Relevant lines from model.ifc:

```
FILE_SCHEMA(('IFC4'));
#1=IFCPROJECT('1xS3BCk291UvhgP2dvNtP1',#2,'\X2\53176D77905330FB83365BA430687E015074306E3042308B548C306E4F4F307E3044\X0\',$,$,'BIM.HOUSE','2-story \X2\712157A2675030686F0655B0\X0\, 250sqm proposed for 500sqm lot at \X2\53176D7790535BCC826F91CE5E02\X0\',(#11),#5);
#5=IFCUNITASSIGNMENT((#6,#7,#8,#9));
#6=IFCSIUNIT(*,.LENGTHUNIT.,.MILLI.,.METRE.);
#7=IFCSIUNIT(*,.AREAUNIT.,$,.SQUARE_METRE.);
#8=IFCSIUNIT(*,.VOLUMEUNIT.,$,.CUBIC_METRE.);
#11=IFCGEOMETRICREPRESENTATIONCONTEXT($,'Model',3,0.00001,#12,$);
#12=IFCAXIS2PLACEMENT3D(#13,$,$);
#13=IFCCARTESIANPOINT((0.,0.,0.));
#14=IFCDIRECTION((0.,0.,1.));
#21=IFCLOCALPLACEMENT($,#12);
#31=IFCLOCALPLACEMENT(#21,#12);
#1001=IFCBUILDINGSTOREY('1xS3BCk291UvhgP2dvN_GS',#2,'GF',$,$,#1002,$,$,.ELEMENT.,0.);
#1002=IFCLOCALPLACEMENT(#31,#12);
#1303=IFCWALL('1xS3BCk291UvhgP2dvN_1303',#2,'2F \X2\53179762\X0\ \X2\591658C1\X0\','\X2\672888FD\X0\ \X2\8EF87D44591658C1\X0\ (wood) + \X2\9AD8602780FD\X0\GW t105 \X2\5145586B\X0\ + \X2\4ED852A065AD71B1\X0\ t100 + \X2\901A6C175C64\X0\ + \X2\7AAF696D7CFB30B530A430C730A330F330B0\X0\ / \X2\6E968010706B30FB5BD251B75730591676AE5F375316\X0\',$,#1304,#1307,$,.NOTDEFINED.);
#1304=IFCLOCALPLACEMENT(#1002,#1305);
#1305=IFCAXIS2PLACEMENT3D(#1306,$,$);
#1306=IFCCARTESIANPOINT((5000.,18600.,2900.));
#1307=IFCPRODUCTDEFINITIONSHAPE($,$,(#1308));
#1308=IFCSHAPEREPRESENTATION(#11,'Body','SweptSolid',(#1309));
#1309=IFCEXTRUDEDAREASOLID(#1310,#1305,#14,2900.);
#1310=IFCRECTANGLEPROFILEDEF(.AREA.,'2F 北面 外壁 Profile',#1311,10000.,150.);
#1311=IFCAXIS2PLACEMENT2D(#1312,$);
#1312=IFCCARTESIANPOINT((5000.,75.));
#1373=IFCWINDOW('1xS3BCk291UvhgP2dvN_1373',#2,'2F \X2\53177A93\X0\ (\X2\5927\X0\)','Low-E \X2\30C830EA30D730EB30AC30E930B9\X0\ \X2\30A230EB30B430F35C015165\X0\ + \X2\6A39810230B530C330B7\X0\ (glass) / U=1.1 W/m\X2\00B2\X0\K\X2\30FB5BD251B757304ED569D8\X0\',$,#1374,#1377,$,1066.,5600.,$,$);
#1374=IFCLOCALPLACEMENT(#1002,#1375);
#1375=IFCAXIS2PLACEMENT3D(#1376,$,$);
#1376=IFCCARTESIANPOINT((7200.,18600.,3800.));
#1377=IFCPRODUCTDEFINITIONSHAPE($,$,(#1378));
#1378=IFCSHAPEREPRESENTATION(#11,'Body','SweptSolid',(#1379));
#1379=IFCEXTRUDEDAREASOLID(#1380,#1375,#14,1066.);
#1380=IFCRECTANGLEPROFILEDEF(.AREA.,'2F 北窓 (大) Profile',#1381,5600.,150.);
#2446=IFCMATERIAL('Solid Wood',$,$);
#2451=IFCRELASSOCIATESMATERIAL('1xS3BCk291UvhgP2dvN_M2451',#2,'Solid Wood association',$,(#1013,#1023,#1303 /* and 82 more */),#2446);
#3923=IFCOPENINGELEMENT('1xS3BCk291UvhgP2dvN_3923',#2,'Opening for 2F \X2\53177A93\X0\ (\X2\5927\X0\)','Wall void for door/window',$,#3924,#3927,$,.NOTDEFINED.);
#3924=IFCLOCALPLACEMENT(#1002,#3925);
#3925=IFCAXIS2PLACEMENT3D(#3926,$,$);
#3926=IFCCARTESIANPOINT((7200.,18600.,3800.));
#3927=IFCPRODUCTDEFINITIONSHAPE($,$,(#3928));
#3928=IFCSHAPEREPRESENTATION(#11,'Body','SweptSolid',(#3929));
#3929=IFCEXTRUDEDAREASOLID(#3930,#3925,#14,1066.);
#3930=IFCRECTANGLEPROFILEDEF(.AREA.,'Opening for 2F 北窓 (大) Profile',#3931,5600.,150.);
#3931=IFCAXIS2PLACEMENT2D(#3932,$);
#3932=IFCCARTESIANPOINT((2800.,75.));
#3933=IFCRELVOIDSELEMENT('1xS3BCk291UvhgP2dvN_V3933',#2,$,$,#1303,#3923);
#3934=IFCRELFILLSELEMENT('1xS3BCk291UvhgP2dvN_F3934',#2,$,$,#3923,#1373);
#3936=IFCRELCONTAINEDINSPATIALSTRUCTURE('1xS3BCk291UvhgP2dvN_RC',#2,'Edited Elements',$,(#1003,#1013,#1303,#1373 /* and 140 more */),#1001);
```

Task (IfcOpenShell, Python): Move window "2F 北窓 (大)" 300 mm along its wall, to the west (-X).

```python
import ifcopenshell
import ifcopenshell.api.geometry
import ifcopenshell.util.placement
import ifcopenshell.util.unit

model = ifcopenshell.open("model.ifc")
unit_scale = ifcopenshell.util.unit.calculate_unit_scale(model)

window = model.by_guid("1xS3BCk291UvhgP2dvN_1373")
opening = window.FillsVoids[0].RelatingOpeningElement
wall = opening.VoidsElements[0].RelatingBuildingElement

wall_matrix = ifcopenshell.util.placement.get_local_placement(wall.ObjectPlacement)
shift = wall_matrix[:3, 0] * -0.3 / unit_scale
before = ifcopenshell.util.placement.get_local_placement(window.ObjectPlacement)[:3, 3].copy()

# The window is not placed relative to its opening, so move both.
for product in (opening, window):
    matrix = ifcopenshell.util.placement.get_local_placement(product.ObjectPlacement)
    matrix[:3, 3] += shift
    ifcopenshell.api.geometry.edit_object_placement(model, product=product, matrix=matrix, is_si=False)

after = ifcopenshell.util.placement.get_local_placement(window.ObjectPlacement)[:3, 3]
print("window moved by", (after - before).round(3) + 0.0)

model.write("model-out.ifc")
```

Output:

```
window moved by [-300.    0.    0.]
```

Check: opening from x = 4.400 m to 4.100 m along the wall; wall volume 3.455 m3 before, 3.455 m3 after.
